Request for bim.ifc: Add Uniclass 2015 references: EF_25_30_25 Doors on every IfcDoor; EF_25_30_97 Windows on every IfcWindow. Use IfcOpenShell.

First a look at what the model holds.

```python
import ifcopenshell

model = ifcopenshell.open("bim.ifc")
print(model.schema)
print("classifications:", [c.Name for c in model.by_type("IfcClassification")])
for ifc_class in ("IfcDoor", "IfcRoof", "IfcStair", "IfcWall", "IfcWindow"):
    print(ifc_class, len(model.by_type(ifc_class)))
```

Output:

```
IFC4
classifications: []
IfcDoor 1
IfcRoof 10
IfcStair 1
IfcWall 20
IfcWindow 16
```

```python
import ifcopenshell
import ifcopenshell.api.classification

model = ifcopenshell.open("bim.ifc")

system = ifcopenshell.api.classification.add_classification(model, classification="Uniclass 2015")

codes = {
    "IfcDoor": ("EF_25_30_25", "Doors"),
    "IfcWindow": ("EF_25_30_97", "Windows"),
}
for ifc_class, (code, name) in codes.items():
    products = model.by_type(ifc_class)
    ifcopenshell.api.classification.add_reference(
        model, products=products, classification=system, identification=code, name=name
    )
    print(code, len(products))

model.write("bim_rev.ifc")
```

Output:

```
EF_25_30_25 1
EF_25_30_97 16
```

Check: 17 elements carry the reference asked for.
